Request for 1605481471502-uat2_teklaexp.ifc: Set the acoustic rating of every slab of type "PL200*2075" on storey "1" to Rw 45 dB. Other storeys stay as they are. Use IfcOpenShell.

First a look at what the model holds.

```python
import ifcopenshell
import ifcopenshell.util.element

model = ifcopenshell.open("1605481471502-uat2_teklaexp.ifc")
print(model.schema)
storey = next(s for s in model.by_type("IfcBuildingStorey") if s.Name == "1")
slabs = [e for e in ifcopenshell.util.element.get_decomposition(storey) if e.is_a("IfcSlab")]
seen = {}
for e in slabs:
    element_type = ifcopenshell.util.element.get_type(e)
    key = (element_type.Name if element_type != e and element_type else None, ifcopenshell.util.element.get_pset(e, "Pset_SlabCommon", "AcousticRating"))
    seen[key] = seen.get(key, 0) + 1
for (name, value), count in sorted(seen.items(), key=str):
    print(count, "x", name, "|", value)
```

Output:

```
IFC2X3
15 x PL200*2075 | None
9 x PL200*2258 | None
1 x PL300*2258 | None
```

```python
import ifcopenshell
import ifcopenshell.api.pset
import ifcopenshell.util.element

model = ifcopenshell.open("1605481471502-uat2_teklaexp.ifc")

storey = next(s for s in model.by_type("IfcBuildingStorey") if s.Name == "1")
slabs = [e for e in ifcopenshell.util.element.get_decomposition(storey) if e.is_a("IfcSlab")]

count = 0
for e in slabs:
    element_type = ifcopenshell.util.element.get_type(e)
    if element_type in (None, e) or element_type.Name != "PL200*2075":
        continue
    found = ifcopenshell.util.element.get_pset(e, "Pset_SlabCommon", should_inherit=False)
    if found:
        pset = model.by_id(found["id"])
        if len(ifcopenshell.util.element.get_elements_by_pset(pset)) > 1:
            pset = ifcopenshell.api.pset.unshare_pset(model, products=[e], pset=pset)[0]
    else:
        pset = ifcopenshell.api.pset.add_pset(model, product=e, name="Pset_SlabCommon")
    ifcopenshell.api.pset.edit_pset(model, pset=pset, properties={"AcousticRating": "Rw 45 dB"})
    count += 1

print(count, "slabs updated")

model.write("1605481471502-uat2_teklaexp_updated.ifc")
```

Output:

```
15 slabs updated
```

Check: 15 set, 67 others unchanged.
